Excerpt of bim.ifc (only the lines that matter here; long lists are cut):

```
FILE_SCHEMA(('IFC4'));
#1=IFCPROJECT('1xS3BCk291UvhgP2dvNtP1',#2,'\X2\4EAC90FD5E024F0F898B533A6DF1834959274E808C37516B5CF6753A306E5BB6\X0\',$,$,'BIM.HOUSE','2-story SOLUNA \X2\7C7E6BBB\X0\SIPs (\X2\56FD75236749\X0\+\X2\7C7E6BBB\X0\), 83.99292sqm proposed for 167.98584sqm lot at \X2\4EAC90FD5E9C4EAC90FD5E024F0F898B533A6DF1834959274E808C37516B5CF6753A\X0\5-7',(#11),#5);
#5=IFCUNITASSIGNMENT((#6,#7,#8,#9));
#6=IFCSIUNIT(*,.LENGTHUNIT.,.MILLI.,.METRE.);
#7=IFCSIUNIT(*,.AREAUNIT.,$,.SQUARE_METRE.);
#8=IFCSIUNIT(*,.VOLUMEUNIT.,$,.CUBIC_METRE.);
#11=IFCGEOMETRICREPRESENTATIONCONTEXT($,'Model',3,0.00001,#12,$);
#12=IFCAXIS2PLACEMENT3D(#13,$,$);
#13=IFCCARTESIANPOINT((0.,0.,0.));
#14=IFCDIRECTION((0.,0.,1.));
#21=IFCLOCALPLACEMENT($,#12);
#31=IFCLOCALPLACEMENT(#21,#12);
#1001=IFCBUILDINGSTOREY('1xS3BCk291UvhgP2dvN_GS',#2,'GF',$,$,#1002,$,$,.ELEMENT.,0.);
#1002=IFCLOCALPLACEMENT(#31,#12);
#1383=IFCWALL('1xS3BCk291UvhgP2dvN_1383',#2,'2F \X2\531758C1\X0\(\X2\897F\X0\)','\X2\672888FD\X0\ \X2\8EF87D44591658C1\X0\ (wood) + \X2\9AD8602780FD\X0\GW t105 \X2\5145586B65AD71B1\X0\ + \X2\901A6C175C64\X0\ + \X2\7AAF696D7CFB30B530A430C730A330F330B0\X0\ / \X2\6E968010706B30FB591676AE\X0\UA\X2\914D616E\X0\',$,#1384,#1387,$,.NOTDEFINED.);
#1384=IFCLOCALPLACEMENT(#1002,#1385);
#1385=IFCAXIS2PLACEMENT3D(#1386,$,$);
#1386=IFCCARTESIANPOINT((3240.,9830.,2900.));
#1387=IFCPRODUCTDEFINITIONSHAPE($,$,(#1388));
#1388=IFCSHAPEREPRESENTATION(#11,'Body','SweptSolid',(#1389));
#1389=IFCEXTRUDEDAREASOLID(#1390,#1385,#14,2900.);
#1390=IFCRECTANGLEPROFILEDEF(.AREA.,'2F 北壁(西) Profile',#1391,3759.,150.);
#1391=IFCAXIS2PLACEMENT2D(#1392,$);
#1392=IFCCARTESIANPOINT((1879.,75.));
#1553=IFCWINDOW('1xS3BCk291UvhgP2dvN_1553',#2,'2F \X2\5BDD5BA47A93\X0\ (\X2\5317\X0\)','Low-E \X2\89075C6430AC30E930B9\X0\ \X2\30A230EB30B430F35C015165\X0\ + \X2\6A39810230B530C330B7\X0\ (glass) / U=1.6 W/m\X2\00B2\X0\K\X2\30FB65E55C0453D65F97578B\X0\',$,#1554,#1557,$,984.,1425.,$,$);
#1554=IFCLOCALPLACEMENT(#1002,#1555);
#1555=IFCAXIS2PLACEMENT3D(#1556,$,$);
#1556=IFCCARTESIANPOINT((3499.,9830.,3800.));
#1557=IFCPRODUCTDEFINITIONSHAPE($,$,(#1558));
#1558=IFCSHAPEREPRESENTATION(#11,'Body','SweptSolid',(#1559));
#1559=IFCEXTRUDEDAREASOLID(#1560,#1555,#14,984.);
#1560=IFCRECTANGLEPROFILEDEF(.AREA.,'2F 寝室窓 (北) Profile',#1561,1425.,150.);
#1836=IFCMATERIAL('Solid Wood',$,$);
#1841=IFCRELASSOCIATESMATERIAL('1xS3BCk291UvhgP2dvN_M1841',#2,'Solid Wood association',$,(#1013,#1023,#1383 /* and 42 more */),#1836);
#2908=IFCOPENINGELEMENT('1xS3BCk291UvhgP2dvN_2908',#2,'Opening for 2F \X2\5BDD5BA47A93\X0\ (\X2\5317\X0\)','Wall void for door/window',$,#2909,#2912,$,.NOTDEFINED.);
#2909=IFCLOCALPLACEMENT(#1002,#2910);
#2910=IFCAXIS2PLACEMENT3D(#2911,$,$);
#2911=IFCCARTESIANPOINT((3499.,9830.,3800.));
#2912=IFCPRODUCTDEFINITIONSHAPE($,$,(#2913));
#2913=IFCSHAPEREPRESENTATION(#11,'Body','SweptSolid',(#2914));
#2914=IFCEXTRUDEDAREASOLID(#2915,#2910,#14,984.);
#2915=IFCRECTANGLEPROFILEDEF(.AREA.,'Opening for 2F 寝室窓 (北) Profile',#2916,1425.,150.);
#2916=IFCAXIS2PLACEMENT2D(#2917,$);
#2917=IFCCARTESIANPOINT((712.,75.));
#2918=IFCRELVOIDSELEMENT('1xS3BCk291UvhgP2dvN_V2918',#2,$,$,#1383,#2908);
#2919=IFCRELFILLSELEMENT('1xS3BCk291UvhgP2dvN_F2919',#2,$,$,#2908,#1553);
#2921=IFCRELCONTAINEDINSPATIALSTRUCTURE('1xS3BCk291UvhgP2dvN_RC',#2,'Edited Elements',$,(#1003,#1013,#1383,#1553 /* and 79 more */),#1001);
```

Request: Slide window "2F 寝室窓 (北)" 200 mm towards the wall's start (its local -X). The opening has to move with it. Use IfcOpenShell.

```python
import ifcopenshell
import ifcopenshell.api.geometry
import ifcopenshell.util.placement
import ifcopenshell.util.unit

model = ifcopenshell.open("bim.ifc")
unit_scale = ifcopenshell.util.unit.calculate_unit_scale(model)

window = model.by_guid("1xS3BCk291UvhgP2dvN_1553")
opening = window.FillsVoids[0].RelatingOpeningElement
wall = opening.VoidsElements[0].RelatingBuildingElement

wall_matrix = ifcopenshell.util.placement.get_local_placement(wall.ObjectPlacement)
shift = wall_matrix[:3, 0] * -0.2 / unit_scale
before = ifcopenshell.util.placement.get_local_placement(window.ObjectPlacement)[:3, 3].copy()

# The window is not placed relative to its opening, so move both.
for product in (opening, window):
    matrix = ifcopenshell.util.placement.get_local_placement(product.ObjectPlacement)
    matrix[:3, 3] += shift
    ifcopenshell.api.geometry.edit_object_placement(model, product=product, matrix=matrix, is_si=False)

after = ifcopenshell.util.placement.get_local_placement(window.ObjectPlacement)[:3, 3]
print("window moved by", (after - before).round(3) + 0.0)

model.write("bim_rev.ifc")
```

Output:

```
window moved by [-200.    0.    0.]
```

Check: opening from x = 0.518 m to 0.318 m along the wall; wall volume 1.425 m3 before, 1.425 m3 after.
